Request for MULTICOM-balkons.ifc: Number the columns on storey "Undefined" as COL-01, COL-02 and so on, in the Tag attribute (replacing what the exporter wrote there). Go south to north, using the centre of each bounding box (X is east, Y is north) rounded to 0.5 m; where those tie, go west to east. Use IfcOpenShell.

First a look at what the model holds.

```python
import ifcopenshell
import ifcopenshell.util.element
import ifcopenshell.util.placement

model = ifcopenshell.open("MULTICOM-balkons.ifc")
print(model.schema)
storey = next(s for s in model.by_type("IfcBuildingStorey") if s.Name == "Undefined")
columns = [e for e in ifcopenshell.util.element.get_decomposition(storey) if e.is_a("IfcColumn")]
for e in sorted(columns, key=lambda e: e.id()):
    origin = ifcopenshell.util.placement.get_local_placement(e.ObjectPlacement)[:3, 3]
    print(e.id(), e.Tag, e.Name, origin.round(2) + 0.0, sep=" | ")
```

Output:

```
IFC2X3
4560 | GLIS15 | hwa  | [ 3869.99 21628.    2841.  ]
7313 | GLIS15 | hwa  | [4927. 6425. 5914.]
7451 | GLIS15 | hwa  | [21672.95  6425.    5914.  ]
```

```python
import ifcopenshell
import ifcopenshell.geom
import ifcopenshell.util.element
import ifcopenshell.util.shape

model = ifcopenshell.open("MULTICOM-balkons.ifc")
settings = ifcopenshell.geom.settings()
settings.set("use-world-coords", True)


def centre(element):
    shape = ifcopenshell.geom.create_shape(settings, element)
    return ifcopenshell.util.shape.get_bbox_centroid(shape.geometry)


storey = next(s for s in model.by_type("IfcBuildingStorey") if s.Name == "Undefined")
columns = [e for e in ifcopenshell.util.element.get_decomposition(storey) if e.is_a("IfcColumn")]

# Insertion points can sit at a corner or the storey origin, so sort by the geometry (in metres).
centres = {e: centre(e) for e in columns}
columns.sort(key=lambda e: (round(centres[e][1] / 0.5), centres[e][0]))

for i, e in enumerate(columns, start=1):
    number = f"COL-{i:02d}"
    e.Tag = number
    print(e.id(), number)

model.write("MULTICOM-balkons_rev.ifc")
```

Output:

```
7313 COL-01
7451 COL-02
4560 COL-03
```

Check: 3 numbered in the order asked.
